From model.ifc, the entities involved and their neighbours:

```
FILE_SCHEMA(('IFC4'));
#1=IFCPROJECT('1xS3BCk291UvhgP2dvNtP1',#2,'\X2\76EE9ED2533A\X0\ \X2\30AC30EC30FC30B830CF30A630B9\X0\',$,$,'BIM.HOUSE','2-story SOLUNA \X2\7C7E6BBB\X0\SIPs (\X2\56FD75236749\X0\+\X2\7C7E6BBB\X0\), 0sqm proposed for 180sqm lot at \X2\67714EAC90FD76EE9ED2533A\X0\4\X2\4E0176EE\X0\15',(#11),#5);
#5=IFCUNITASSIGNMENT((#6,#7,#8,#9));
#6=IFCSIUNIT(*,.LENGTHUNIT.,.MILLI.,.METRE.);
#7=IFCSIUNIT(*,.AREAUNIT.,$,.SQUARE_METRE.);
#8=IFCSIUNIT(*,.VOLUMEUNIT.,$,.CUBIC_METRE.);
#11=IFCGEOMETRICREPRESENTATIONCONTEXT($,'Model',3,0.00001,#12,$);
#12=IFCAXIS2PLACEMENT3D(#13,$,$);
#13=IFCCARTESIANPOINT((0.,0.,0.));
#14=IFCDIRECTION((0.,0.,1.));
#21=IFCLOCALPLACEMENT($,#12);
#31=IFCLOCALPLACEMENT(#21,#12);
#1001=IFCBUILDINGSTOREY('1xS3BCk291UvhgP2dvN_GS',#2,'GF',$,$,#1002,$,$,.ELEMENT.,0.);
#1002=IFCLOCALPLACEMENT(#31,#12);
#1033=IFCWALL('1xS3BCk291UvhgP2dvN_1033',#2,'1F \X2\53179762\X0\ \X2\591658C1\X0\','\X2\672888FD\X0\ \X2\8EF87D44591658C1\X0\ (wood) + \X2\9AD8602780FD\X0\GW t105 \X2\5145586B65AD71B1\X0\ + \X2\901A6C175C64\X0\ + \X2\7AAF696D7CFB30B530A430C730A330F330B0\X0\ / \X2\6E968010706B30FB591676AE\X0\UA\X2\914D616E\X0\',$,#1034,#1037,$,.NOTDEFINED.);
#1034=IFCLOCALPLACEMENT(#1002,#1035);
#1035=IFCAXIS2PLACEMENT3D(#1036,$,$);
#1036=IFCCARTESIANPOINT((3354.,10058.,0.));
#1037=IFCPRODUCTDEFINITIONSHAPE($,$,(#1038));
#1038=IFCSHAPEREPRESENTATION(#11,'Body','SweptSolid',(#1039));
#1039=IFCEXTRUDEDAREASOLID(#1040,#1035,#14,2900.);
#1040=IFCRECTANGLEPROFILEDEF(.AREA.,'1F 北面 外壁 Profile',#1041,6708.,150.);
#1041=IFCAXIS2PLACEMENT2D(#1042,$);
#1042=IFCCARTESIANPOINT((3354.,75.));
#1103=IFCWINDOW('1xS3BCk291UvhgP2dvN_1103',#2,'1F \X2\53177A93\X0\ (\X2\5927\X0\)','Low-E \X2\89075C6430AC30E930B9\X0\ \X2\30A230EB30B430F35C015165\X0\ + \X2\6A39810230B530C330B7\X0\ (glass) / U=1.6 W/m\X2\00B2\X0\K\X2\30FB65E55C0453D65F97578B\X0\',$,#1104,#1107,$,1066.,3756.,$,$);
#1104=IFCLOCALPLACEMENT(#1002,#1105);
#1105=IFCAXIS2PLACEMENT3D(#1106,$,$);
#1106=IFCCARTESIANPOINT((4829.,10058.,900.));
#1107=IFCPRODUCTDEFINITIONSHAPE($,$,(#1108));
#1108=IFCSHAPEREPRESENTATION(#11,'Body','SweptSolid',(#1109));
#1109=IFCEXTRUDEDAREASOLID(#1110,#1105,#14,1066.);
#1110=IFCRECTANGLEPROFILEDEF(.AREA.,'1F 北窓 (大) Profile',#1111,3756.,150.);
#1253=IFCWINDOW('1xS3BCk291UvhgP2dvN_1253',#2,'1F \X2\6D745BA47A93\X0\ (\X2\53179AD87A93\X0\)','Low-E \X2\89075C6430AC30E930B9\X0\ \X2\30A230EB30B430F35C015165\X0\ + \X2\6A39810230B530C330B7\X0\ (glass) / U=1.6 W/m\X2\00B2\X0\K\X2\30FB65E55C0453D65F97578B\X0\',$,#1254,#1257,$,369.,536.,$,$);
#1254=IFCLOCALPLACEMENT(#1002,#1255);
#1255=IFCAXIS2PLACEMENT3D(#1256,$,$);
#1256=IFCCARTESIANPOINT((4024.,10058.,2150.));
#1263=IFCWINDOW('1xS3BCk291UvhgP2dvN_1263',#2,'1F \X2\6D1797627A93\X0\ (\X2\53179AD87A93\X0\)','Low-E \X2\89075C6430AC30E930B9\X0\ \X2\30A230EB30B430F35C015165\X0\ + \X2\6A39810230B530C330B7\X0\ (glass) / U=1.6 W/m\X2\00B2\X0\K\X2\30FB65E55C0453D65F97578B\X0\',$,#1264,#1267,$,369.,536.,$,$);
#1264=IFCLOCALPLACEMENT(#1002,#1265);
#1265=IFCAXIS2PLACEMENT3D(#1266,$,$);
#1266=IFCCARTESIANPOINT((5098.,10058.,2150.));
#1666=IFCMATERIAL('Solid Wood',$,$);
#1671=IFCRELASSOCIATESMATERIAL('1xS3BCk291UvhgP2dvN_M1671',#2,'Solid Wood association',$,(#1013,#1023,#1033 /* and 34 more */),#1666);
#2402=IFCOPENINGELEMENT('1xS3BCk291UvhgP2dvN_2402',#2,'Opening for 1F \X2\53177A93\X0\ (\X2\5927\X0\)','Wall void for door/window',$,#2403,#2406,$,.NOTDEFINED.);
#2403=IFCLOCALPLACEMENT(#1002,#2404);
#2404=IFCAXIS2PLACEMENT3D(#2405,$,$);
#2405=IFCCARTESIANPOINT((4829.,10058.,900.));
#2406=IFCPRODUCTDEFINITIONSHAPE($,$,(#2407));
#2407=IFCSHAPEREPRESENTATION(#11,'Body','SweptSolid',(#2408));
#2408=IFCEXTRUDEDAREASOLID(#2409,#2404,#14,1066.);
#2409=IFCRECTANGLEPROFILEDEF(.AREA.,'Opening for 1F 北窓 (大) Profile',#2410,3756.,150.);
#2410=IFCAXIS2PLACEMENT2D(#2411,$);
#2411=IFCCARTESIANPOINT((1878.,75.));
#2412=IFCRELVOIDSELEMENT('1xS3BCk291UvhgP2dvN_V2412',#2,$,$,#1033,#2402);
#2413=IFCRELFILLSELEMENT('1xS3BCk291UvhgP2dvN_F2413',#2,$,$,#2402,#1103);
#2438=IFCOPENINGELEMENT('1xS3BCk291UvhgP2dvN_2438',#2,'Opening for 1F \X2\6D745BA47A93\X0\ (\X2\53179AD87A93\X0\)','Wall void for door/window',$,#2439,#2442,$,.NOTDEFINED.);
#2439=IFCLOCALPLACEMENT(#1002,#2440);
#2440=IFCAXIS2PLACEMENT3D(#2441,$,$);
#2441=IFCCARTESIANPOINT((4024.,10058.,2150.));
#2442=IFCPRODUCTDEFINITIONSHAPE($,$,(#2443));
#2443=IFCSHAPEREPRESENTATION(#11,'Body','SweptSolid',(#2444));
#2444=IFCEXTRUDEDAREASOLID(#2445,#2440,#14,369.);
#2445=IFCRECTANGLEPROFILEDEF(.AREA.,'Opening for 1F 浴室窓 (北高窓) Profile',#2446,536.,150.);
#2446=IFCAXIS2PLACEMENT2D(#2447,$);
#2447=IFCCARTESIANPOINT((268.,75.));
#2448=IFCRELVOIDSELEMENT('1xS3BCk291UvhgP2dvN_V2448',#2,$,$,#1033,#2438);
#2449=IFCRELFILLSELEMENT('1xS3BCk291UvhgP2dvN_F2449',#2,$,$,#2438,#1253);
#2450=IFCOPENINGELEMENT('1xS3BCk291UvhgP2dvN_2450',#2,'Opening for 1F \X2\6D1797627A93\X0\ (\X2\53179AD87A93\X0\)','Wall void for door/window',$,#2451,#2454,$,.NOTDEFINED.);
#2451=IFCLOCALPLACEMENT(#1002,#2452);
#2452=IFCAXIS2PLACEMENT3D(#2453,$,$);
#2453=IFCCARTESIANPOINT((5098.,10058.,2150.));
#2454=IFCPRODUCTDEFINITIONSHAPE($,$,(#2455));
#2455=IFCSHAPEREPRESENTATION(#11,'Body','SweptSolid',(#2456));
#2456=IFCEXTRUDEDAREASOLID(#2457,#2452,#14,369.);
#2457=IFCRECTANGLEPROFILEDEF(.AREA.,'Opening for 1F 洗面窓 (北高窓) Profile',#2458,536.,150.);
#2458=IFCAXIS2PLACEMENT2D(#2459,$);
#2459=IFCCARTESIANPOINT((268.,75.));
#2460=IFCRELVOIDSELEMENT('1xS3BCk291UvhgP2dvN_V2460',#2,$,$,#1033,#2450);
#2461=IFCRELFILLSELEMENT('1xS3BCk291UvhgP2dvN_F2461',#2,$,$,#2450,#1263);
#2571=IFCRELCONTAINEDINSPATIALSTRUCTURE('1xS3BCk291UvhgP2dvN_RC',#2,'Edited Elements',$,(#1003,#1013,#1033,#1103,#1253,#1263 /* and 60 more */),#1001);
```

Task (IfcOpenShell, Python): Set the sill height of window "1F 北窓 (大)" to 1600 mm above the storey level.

```python
import numpy as np
import ifcopenshell
import ifcopenshell.api.geometry
import ifcopenshell.geom
import ifcopenshell.util.element
import ifcopenshell.util.placement
import ifcopenshell.util.shape
import ifcopenshell.util.unit

model = ifcopenshell.open("model.ifc")
unit_scale = ifcopenshell.util.unit.calculate_unit_scale(model)

window = model.by_guid("1xS3BCk291UvhgP2dvN_1103")
opening = window.FillsVoids[0].RelatingOpeningElement
storey = ifcopenshell.util.element.get_container(window, ifc_class="IfcBuildingStorey")
level = ifcopenshell.util.placement.get_local_placement(storey.ObjectPlacement)[2, 3]

# The opening's origin need not be at the sill, so measure its lowest point.
shape = ifcopenshell.geom.create_shape(ifcopenshell.geom.settings(), opening)
bottom = ifcopenshell.util.shape.get_shape_bottom_elevation(shape, shape.geometry) / unit_scale
dz = level + 1600.0 - bottom

shift = np.array([0.0, 0.0, dz])
# The window is not placed relative to its opening, so move both.
for product in (opening, window):
    matrix = ifcopenshell.util.placement.get_local_placement(product.ObjectPlacement)
    matrix[:3, 3] += shift
    ifcopenshell.api.geometry.edit_object_placement(model, product=product, matrix=matrix, is_si=False)

print(f"moved by {dz * unit_scale:+.3f} m")

model.write("model_rev.ifc")
```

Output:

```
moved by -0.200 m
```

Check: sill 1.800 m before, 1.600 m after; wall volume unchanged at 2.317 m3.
